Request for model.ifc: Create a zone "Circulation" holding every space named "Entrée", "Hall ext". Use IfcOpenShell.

First a look at what the model holds.

```python
import ifcopenshell

model = ifcopenshell.open("model.ifc")
print(model.schema)
seen = {}
for space in model.by_type("IfcSpace"):
    seen[space.LongName] = seen.get(space.LongName, 0) + 1
for name, count in sorted(seen.items(), key=str):
    print(count, "x", name)
print("zones:", [z.Name for z in model.by_type("IfcZone")][:20])
```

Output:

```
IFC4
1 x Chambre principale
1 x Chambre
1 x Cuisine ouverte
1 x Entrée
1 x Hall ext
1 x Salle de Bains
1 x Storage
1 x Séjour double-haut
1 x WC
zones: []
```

```python
import ifcopenshell
import ifcopenshell.api.group
import ifcopenshell.api.root

model = ifcopenshell.open("model.ifc")

names = {"Entrée", "Hall ext"}
spaces = [s for s in model.by_type("IfcSpace") if s.LongName in names]

zone = ifcopenshell.api.root.create_entity(model, ifc_class="IfcZone", name="Circulation")
ifcopenshell.api.group.assign_group(model, products=spaces, group=zone)
print(len(spaces), "spaces in", zone.Name)

model.write("model_edited.ifc")
```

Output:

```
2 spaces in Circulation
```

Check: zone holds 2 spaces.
